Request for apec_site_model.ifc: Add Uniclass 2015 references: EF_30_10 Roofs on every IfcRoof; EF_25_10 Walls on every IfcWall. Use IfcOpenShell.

First a look at what the model holds.

```python
import ifcopenshell

model = ifcopenshell.open("apec_site_model.ifc")
print(model.schema)
print("classifications:", [c.Name for c in model.by_type("IfcClassification")])
for ifc_class in ("IfcDoor", "IfcRoof", "IfcStair", "IfcWall", "IfcWindow"):
    print(ifc_class, len(model.by_type(ifc_class)))
```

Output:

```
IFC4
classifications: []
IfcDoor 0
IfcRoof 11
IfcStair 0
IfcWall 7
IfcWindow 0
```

```python
import ifcopenshell
import ifcopenshell.api.classification

model = ifcopenshell.open("apec_site_model.ifc")

system = ifcopenshell.api.classification.add_classification(model, classification="Uniclass 2015")

codes = {
    "IfcRoof": ("EF_30_10", "Roofs"),
    "IfcWall": ("EF_25_10", "Walls"),
}
for ifc_class, (code, name) in codes.items():
    products = model.by_type(ifc_class)
    ifcopenshell.api.classification.add_reference(
        model, products=products, classification=system, identification=code, name=name
    )
    print(code, len(products))

model.write("apec_site_model_v2.ifc")
```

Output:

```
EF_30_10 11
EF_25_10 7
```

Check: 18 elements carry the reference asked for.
